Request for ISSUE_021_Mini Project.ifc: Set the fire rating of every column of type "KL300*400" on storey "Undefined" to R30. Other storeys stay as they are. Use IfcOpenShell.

First a look at what the model holds.

```python
import ifcopenshell
import ifcopenshell.util.element

model = ifcopenshell.open("ISSUE_021_Mini Project.ifc")
print(model.schema)
storey = next(s for s in model.by_type("IfcBuildingStorey") if s.Name == "Undefined")
columns = [e for e in ifcopenshell.util.element.get_decomposition(storey) if e.is_a("IfcColumn")]
seen = {}
for e in columns:
    element_type = ifcopenshell.util.element.get_type(e)
    key = (element_type.Name if element_type != e and element_type else None, ifcopenshell.util.element.get_pset(e, "Pset_ColumnCommon", "FireRating"))
    seen[key] = seen.get(key, 0) + 1
for (name, value), count in sorted(seen.items(), key=str):
    print(count, "x", name, "|", value)
```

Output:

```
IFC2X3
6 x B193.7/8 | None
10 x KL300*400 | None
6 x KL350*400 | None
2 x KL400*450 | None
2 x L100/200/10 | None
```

```python
import ifcopenshell
import ifcopenshell.api.pset
import ifcopenshell.util.element

model = ifcopenshell.open("ISSUE_021_Mini Project.ifc")

storey = next(s for s in model.by_type("IfcBuildingStorey") if s.Name == "Undefined")
columns = [e for e in ifcopenshell.util.element.get_decomposition(storey) if e.is_a("IfcColumn")]

count = 0
for e in columns:
    element_type = ifcopenshell.util.element.get_type(e)
    if element_type in (None, e) or element_type.Name != "KL300*400":
        continue
    found = ifcopenshell.util.element.get_pset(e, "Pset_ColumnCommon", should_inherit=False)
    if found:
        pset = model.by_id(found["id"])
        if len(ifcopenshell.util.element.get_elements_by_pset(pset)) > 1:
            pset = ifcopenshell.api.pset.unshare_pset(model, products=[e], pset=pset)[0]
    else:
        pset = ifcopenshell.api.pset.add_pset(model, product=e, name="Pset_ColumnCommon")
    ifcopenshell.api.pset.edit_pset(model, pset=pset, properties={"FireRating": "R30"})
    count += 1

print(count, "columns updated")

model.write("ISSUE_021_Mini Project_rev.ifc")
```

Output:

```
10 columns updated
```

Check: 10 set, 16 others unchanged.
